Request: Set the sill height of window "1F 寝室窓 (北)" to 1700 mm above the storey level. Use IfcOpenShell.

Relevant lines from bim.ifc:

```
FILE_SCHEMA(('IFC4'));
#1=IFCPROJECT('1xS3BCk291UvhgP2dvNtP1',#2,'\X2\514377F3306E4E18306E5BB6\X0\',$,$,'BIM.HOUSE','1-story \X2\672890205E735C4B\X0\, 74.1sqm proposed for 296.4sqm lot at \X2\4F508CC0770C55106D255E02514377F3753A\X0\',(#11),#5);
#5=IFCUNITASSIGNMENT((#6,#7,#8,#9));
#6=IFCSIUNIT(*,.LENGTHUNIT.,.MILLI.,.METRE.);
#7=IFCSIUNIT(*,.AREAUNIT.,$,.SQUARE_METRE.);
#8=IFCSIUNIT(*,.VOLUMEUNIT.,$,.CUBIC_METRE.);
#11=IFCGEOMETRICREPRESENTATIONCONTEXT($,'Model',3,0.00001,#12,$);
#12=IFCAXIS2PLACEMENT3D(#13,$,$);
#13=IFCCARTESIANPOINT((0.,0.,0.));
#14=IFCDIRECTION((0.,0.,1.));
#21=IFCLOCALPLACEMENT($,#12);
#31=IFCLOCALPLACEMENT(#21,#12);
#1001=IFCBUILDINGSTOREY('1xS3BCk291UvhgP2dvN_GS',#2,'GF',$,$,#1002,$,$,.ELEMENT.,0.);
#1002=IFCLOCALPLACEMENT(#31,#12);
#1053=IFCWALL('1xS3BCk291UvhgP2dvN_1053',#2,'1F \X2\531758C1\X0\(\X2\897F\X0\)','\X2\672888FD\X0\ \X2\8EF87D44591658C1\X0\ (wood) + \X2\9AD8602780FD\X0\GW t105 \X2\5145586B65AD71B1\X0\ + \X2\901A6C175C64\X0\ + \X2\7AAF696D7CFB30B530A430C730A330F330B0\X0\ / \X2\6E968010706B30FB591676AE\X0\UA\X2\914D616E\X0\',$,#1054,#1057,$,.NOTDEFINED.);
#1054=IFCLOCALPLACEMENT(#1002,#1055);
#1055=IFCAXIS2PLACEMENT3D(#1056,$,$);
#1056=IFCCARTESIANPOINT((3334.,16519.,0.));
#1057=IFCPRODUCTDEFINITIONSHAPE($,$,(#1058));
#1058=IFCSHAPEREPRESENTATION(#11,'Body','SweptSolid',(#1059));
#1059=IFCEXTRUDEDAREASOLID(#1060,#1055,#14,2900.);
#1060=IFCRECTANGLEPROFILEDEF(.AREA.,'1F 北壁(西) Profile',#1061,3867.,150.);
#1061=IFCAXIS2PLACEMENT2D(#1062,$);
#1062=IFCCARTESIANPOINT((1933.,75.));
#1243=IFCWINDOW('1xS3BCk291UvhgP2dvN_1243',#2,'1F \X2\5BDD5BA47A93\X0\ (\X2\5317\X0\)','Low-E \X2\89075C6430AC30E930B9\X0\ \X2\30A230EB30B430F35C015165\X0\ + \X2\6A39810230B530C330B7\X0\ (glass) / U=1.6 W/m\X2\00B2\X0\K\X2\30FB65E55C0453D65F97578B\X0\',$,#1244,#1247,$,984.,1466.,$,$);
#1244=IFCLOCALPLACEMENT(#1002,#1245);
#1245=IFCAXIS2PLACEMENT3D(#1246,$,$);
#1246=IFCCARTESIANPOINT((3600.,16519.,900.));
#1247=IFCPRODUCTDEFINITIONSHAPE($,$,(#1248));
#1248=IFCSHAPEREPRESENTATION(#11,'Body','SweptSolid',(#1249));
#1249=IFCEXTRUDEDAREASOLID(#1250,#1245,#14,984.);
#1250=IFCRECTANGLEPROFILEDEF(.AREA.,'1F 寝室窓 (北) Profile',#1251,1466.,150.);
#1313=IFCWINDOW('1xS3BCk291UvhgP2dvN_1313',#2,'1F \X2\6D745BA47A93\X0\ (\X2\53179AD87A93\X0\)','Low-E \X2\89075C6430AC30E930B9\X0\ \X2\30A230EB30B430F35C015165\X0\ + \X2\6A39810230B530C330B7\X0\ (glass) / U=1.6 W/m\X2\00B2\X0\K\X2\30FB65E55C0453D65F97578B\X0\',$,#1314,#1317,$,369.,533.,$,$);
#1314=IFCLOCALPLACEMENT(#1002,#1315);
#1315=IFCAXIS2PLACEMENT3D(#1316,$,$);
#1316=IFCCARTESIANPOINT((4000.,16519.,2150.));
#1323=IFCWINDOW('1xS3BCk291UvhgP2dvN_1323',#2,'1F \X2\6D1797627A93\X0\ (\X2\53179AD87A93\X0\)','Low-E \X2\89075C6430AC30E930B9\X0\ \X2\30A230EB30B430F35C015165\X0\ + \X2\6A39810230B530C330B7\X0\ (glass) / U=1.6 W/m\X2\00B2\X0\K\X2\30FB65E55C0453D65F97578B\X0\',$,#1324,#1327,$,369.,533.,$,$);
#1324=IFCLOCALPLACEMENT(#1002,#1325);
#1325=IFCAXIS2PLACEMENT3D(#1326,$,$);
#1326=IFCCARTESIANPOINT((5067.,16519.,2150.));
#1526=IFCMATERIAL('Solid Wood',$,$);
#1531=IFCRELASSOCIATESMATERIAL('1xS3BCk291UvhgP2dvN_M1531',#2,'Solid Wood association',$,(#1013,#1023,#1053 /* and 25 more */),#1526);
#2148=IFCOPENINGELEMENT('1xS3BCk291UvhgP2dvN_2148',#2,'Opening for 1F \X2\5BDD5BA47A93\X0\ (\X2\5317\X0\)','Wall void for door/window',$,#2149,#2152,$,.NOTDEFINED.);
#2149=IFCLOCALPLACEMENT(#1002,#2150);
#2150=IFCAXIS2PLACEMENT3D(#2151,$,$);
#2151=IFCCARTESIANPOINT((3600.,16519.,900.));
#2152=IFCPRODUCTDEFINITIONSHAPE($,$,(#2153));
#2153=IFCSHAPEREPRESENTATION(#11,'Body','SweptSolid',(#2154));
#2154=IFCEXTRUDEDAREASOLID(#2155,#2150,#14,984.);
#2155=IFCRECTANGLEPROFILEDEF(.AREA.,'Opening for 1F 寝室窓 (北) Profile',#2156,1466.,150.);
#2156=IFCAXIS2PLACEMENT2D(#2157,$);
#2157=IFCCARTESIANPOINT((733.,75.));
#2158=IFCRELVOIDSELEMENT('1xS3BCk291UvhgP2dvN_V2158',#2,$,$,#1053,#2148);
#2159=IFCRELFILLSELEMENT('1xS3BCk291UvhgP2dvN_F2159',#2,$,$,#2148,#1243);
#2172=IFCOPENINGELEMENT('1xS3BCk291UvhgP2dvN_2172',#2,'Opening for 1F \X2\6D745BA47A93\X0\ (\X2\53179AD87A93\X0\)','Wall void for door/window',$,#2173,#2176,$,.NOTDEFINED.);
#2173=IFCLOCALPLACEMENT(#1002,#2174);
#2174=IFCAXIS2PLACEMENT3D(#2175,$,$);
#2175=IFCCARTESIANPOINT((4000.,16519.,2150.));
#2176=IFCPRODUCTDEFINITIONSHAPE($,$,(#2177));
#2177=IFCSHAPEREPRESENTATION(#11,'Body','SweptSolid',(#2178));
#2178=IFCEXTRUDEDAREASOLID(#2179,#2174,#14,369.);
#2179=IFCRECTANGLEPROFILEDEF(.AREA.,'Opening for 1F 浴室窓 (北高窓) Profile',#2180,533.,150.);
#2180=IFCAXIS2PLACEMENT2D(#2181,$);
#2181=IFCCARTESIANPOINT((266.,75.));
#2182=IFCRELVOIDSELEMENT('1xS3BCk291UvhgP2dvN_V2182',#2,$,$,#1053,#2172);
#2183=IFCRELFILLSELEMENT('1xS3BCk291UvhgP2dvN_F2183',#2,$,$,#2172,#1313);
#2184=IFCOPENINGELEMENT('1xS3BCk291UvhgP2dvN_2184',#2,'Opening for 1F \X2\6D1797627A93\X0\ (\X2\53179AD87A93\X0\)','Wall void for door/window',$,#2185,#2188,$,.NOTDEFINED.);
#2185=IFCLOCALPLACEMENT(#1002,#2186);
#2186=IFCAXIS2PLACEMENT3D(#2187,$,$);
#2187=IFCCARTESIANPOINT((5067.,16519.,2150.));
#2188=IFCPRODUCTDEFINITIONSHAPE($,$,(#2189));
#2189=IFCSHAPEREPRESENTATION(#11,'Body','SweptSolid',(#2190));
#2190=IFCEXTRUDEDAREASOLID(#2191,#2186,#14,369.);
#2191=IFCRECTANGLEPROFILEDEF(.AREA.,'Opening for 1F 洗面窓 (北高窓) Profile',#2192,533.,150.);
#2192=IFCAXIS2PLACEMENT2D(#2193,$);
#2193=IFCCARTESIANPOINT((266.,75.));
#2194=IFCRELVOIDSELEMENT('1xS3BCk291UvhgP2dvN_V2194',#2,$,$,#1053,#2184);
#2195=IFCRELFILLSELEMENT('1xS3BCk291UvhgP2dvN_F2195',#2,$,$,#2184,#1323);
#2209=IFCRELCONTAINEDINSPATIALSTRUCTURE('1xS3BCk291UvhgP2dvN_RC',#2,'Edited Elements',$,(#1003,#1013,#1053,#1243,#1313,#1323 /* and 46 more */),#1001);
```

```python
import numpy as np
import ifcopenshell
import ifcopenshell.api.geometry
import ifcopenshell.geom
import ifcopenshell.util.element
import ifcopenshell.util.placement
import ifcopenshell.util.shape
import ifcopenshell.util.unit

model = ifcopenshell.open("bim.ifc")
unit_scale = ifcopenshell.util.unit.calculate_unit_scale(model)

window = model.by_id(1243)
opening = window.FillsVoids[0].RelatingOpeningElement
storey = ifcopenshell.util.element.get_container(window, ifc_class="IfcBuildingStorey")
level = ifcopenshell.util.placement.get_local_placement(storey.ObjectPlacement)[2, 3]

# The opening's origin need not be at the sill, so measure its lowest point.
shape = ifcopenshell.geom.create_shape(ifcopenshell.geom.settings(), opening)
bottom = ifcopenshell.util.shape.get_shape_bottom_elevation(shape, shape.geometry) / unit_scale
dz = level + 1.7 / unit_scale - bottom

shift = np.array([0.0, 0.0, dz])
# The window is not placed relative to its opening, so move both.
for product in (opening, window):
    matrix = ifcopenshell.util.placement.get_local_placement(product.ObjectPlacement)
    matrix[:3, 3] += shift
    ifcopenshell.api.geometry.edit_object_placement(model, product=product, matrix=matrix, is_si=False)

print(f"moved by {dz * unit_scale:+.3f} m")

model.write("bim-out.ifc")
```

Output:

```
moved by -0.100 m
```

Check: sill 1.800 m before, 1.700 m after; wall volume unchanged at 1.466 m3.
